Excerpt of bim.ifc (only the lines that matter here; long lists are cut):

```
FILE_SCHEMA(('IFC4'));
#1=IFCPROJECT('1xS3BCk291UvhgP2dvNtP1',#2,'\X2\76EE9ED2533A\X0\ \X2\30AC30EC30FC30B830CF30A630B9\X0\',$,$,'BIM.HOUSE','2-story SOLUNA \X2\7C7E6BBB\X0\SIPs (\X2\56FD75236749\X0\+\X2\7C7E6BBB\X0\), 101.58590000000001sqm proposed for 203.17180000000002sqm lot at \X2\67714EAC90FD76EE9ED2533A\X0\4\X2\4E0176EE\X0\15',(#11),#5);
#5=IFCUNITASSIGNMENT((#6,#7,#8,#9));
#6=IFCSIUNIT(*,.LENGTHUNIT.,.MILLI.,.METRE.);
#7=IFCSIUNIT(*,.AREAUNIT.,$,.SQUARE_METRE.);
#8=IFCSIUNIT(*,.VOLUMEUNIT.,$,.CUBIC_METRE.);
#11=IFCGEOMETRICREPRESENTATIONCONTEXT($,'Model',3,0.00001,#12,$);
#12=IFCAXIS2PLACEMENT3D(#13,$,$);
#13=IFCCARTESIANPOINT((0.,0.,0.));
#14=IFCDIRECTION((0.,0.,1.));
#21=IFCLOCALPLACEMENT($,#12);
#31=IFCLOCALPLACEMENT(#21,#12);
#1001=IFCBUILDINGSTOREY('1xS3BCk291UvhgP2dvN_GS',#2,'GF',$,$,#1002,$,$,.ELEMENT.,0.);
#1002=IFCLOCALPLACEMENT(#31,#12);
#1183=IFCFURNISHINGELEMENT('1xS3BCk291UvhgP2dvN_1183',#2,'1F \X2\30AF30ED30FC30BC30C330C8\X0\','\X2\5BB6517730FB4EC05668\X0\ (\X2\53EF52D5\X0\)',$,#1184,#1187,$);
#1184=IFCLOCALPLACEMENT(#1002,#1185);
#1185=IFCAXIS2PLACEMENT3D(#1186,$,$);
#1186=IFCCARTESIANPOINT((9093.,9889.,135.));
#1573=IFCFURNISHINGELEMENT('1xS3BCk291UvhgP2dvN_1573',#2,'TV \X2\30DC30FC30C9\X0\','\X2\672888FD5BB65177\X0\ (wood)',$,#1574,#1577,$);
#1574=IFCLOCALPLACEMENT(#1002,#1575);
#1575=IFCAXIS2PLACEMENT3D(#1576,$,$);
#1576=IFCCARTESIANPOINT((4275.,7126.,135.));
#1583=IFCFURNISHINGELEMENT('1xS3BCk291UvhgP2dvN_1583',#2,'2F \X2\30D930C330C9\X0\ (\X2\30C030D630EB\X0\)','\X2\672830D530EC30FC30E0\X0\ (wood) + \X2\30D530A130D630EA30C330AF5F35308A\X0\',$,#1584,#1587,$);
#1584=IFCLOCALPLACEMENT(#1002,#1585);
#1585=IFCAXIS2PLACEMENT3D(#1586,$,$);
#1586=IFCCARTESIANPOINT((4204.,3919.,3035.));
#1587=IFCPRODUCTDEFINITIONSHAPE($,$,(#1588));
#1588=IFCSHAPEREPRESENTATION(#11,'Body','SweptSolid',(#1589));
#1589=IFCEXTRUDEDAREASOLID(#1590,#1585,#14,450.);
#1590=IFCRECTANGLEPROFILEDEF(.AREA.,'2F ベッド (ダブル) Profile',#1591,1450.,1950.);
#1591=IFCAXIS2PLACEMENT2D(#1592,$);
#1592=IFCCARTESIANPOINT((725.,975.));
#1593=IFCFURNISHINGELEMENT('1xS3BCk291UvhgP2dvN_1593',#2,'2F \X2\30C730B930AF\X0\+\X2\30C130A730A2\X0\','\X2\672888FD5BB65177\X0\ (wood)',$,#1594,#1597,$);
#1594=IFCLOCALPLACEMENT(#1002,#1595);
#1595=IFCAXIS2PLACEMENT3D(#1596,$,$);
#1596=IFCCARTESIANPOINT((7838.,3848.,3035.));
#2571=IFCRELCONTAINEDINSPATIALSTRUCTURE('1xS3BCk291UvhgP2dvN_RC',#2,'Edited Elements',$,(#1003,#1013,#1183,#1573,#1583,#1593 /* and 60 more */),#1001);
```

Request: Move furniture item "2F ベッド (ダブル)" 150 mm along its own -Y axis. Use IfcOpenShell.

```python
import ifcopenshell
import ifcopenshell.api.geometry
import ifcopenshell.util.placement

model = ifcopenshell.open("bim.ifc")

item = model.by_guid("1xS3BCk291UvhgP2dvN_1583")
matrix = ifcopenshell.util.placement.get_local_placement(item.ObjectPlacement)
matrix[:3, 3] -= matrix[:3, 1] * 150.0
ifcopenshell.api.geometry.edit_object_placement(model, product=item, matrix=matrix, is_si=False)

print(ifcopenshell.util.placement.get_local_placement(item.ObjectPlacement).round(3) + 0.0)

model.write("bim_updated.ifc")
```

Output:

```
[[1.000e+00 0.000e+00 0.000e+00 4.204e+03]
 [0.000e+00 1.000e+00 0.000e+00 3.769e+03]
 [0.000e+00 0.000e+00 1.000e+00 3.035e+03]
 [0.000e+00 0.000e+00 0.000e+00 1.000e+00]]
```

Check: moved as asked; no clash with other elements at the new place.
